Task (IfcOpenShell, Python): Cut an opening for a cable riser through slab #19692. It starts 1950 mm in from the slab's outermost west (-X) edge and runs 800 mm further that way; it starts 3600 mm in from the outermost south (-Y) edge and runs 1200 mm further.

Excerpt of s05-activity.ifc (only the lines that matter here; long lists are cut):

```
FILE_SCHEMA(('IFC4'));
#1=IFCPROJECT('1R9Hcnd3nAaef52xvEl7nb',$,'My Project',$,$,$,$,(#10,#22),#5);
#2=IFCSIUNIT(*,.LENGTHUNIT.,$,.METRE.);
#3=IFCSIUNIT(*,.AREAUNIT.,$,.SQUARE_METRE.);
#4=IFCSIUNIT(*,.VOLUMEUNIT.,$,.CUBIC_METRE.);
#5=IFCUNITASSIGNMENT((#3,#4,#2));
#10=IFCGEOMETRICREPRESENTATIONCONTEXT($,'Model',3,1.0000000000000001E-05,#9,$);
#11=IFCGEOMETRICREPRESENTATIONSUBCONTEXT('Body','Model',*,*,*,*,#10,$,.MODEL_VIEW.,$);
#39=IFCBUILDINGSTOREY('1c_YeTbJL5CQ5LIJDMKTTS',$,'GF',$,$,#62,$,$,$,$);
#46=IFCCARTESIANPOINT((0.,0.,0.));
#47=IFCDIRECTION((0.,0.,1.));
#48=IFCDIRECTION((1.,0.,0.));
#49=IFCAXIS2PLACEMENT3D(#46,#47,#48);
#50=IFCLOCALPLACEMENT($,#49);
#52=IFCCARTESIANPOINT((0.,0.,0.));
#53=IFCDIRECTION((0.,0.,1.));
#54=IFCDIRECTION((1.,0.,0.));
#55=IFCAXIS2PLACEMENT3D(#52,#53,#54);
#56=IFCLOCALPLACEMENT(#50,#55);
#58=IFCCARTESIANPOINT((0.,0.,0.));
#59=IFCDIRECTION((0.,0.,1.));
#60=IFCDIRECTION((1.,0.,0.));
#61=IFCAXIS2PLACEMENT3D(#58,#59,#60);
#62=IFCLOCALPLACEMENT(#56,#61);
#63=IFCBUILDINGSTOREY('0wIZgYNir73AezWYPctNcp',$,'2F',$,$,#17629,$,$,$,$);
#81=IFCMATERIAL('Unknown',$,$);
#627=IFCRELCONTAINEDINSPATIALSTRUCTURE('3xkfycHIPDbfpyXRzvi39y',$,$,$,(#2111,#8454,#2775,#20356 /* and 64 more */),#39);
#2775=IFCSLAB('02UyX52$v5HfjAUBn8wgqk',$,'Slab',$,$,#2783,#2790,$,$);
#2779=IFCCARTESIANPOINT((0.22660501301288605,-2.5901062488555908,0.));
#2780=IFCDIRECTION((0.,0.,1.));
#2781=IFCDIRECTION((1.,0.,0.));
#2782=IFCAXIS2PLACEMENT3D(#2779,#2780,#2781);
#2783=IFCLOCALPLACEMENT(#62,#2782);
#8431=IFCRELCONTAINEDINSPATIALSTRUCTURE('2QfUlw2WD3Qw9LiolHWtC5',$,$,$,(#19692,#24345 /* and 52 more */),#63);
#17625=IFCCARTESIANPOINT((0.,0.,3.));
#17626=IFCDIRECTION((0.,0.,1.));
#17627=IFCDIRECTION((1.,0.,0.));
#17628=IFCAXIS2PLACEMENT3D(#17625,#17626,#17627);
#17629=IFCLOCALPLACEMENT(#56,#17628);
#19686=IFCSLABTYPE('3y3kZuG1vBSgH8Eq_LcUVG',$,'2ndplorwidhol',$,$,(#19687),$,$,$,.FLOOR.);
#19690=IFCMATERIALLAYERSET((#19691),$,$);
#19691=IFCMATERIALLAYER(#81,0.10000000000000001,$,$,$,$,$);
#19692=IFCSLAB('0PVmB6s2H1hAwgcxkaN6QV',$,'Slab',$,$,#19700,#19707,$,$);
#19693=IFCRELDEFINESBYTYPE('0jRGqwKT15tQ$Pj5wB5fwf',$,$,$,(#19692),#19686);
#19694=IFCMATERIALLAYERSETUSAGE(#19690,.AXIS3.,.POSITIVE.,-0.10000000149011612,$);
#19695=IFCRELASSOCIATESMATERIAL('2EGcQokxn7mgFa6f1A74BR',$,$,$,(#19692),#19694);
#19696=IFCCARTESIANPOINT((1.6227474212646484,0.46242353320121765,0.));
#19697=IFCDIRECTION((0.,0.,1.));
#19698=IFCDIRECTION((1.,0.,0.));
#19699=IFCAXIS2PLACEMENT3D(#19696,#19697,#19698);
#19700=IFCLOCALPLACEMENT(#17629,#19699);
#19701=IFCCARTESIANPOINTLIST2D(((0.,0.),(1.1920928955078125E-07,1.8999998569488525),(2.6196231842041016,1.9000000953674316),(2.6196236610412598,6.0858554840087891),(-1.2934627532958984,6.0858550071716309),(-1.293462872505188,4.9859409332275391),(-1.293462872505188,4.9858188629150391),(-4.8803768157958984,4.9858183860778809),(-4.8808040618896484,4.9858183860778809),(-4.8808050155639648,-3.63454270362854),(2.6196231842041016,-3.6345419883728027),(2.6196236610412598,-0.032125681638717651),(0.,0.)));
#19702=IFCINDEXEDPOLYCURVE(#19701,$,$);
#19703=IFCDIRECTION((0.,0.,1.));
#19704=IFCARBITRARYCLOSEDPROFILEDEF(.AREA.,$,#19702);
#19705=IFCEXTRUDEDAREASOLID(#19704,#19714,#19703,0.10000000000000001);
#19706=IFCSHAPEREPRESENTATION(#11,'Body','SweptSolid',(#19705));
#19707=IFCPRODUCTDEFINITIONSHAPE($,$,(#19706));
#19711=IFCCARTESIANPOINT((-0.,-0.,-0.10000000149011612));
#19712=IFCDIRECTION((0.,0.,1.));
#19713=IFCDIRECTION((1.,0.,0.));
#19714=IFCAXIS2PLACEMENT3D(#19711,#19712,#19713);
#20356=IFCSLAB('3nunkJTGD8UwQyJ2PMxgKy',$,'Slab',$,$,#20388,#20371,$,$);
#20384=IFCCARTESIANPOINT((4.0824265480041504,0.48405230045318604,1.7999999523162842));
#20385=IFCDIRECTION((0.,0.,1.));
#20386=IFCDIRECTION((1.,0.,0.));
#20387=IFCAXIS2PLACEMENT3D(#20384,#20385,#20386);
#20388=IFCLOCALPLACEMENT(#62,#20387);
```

```python
import numpy as np
import ifcopenshell
import ifcopenshell.api.feature
import ifcopenshell.api.geometry
import ifcopenshell.api.root
import ifcopenshell.geom
import ifcopenshell.util.placement
import ifcopenshell.util.representation
import ifcopenshell.util.shape
import ifcopenshell.util.unit

model = ifcopenshell.open("s05-activity.ifc")
unit_scale = ifcopenshell.util.unit.calculate_unit_scale(model)
settings = ifcopenshell.geom.settings()


def volume(element):
    """Net volume in cubic metres, openings subtracted."""
    shape = ifcopenshell.geom.create_shape(settings, element)
    return ifcopenshell.util.shape.get_volume(shape.geometry)


slab = model.by_id(19692)
before = volume(slab)

# Extent in the slab's own axes, in metres. The edges named are its -X and -Y sides.
slab_shape = ifcopenshell.geom.create_shape(settings, slab)
vertices = ifcopenshell.util.shape.get_vertices(slab_shape.geometry)
x_min, y_min, bottom = vertices.min(axis=0)
top = vertices[:, 2].max()

opening = ifcopenshell.api.root.create_entity(model, ifc_class="IfcOpeningElement", name="Cable riser opening", predefined_type="OPENING")
context = ifcopenshell.util.representation.get_context(model, "Model", "Body", "MODEL_VIEW")
width, depth = 0.8, 1.2
outline = [(0.0, 0.0), (width, 0.0), (width, depth), (0.0, depth), (0.0, 0.0)]
# Overshoot both faces by 50 mm so the cut is clean.
shape = ifcopenshell.api.geometry.add_slab_representation(
    model, context=context, depth=top - bottom + 0.1, polyline=outline
)
ifcopenshell.api.geometry.assign_representation(model, product=opening, representation=shape)

matrix = ifcopenshell.util.placement.get_local_placement(slab.ObjectPlacement)
matrix[:, 3] = matrix @ np.append(np.array([x_min + 1.95, y_min + 3.6, bottom - 0.05]) / unit_scale, 1.0)
ifcopenshell.api.geometry.edit_object_placement(model, product=opening, matrix=matrix, is_si=False)
ifcopenshell.api.feature.add_feature(model, feature=opening, element=slab)

after = volume(slab)

print(f"slab volume {before:.3f} -> {after:.3f} m3")

model.write("s05-activity_v2.ifc")
```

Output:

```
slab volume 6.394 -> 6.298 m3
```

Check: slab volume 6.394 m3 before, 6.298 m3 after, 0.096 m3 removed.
